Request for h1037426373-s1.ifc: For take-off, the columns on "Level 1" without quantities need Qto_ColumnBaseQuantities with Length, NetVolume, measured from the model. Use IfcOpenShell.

First a look at what the model holds.

```python
import ifcopenshell
import ifcopenshell.util.element
import ifcopenshell.util.unit

model = ifcopenshell.open("h1037426373-s1.ifc")
print(model.schema)
for unit_type in ("LENGTHUNIT", "AREAUNIT", "VOLUMEUNIT"):
    print(unit_type, ifcopenshell.util.unit.calculate_unit_scale(model, unit_type))
storey = next(s for s in model.by_type("IfcBuildingStorey") if s.Name == "Level 1")
columns = [e for e in ifcopenshell.util.element.get_decomposition(storey) if e.is_a("IfcColumn")]
for e in sorted(columns, key=lambda e: e.id()):
    print(e.id(), e.is_a(), e.Name, list(ifcopenshell.util.element.get_psets(e, qtos_only=True)), sep=" | ")
```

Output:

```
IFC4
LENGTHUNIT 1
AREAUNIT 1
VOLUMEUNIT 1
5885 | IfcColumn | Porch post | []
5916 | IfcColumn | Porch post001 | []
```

```python
import ifcopenshell
import ifcopenshell.api.pset
import ifcopenshell.geom
import ifcopenshell.util.element
import ifcopenshell.util.shape
import ifcopenshell.util.unit

model = ifcopenshell.open("h1037426373-s1.ifc")
unit_scale = ifcopenshell.util.unit.calculate_unit_scale(model)
volume_scale = ifcopenshell.util.unit.calculate_unit_scale(model, "VOLUMEUNIT")
settings = ifcopenshell.geom.settings()

storey = next(s for s in model.by_type("IfcBuildingStorey") if s.Name == "Level 1")
columns = [e for e in ifcopenshell.util.element.get_decomposition(storey) if e.is_a("IfcColumn")]

for e in sorted(columns, key=lambda e: e.id()):
    if ifcopenshell.util.element.get_psets(e, qtos_only=True, should_inherit=False):
        continue
    # Geometry comes back in metres, in the element's own axes.
    shape = ifcopenshell.geom.create_shape(settings, e)
    values = {
        "Length": ifcopenshell.util.shape.get_z(shape.geometry) / unit_scale,
        "NetVolume": ifcopenshell.util.shape.get_volume(shape.geometry) / volume_scale,
    }
    qto = ifcopenshell.api.pset.add_qto(model, product=e, name="Qto_ColumnBaseQuantities")
    ifcopenshell.api.pset.edit_qto(model, qto=qto, properties=values)
    print(e.id(), {k: round(v, 3) for k, v in values.items()})

model.write("h1037426373-s1_edited.ifc")
```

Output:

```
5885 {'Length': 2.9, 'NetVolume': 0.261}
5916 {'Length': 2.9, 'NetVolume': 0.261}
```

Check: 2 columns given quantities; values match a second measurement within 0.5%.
